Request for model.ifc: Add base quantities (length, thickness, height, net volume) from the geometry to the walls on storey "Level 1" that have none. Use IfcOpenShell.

First a look at what the model holds.

```python
import ifcopenshell
import ifcopenshell.util.element
import ifcopenshell.util.unit

model = ifcopenshell.open("model.ifc")
print(model.schema)
for unit_type in ("LENGTHUNIT", "AREAUNIT", "VOLUMEUNIT"):
    print(unit_type, ifcopenshell.util.unit.calculate_unit_scale(model, unit_type))
storey = next(s for s in model.by_type("IfcBuildingStorey") if s.Name == "Level 1")
walls = [e for e in ifcopenshell.util.element.get_decomposition(storey) if e.is_a("IfcWall")]
for e in sorted(walls, key=lambda e: e.id()):
    print(e.id(), e.is_a(), e.Name, list(ifcopenshell.util.element.get_psets(e, qtos_only=True)), sep=" | ")
```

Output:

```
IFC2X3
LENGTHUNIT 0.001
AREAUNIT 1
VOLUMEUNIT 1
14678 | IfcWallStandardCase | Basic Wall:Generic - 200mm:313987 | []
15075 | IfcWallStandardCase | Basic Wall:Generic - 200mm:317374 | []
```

```python
import ifcopenshell
import ifcopenshell.api.pset
import ifcopenshell.geom
import ifcopenshell.util.element
import ifcopenshell.util.shape
import ifcopenshell.util.unit

model = ifcopenshell.open("model.ifc")
unit_scale = ifcopenshell.util.unit.calculate_unit_scale(model)
volume_scale = ifcopenshell.util.unit.calculate_unit_scale(model, "VOLUMEUNIT")
settings = ifcopenshell.geom.settings()

storey = next(s for s in model.by_type("IfcBuildingStorey") if s.Name == "Level 1")
walls = [e for e in ifcopenshell.util.element.get_decomposition(storey) if e.is_a("IfcWall")]

for e in sorted(walls, key=lambda e: e.id()):
    if ifcopenshell.util.element.get_psets(e, qtos_only=True, should_inherit=False):
        continue
    # Geometry comes back in metres, in the element's own axes.
    shape = ifcopenshell.geom.create_shape(settings, e)
    values = {
        "Length": ifcopenshell.util.shape.get_x(shape.geometry) / unit_scale,
        "Width": ifcopenshell.util.shape.get_y(shape.geometry) / unit_scale,
        "Height": ifcopenshell.util.shape.get_z(shape.geometry) / unit_scale,
        "NetVolume": ifcopenshell.util.shape.get_volume(shape.geometry) / volume_scale,
    }
    qto = ifcopenshell.api.pset.add_qto(model, product=e, name="BaseQuantities")
    ifcopenshell.api.pset.edit_qto(model, qto=qto, properties=values)
    print(e.id(), {k: round(v, 3) for k, v in values.items()})

model.write("model-out.ifc")
```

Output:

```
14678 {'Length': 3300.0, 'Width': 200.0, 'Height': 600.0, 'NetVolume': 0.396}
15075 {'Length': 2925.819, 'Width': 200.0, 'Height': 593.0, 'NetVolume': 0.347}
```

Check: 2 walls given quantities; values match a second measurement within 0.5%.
